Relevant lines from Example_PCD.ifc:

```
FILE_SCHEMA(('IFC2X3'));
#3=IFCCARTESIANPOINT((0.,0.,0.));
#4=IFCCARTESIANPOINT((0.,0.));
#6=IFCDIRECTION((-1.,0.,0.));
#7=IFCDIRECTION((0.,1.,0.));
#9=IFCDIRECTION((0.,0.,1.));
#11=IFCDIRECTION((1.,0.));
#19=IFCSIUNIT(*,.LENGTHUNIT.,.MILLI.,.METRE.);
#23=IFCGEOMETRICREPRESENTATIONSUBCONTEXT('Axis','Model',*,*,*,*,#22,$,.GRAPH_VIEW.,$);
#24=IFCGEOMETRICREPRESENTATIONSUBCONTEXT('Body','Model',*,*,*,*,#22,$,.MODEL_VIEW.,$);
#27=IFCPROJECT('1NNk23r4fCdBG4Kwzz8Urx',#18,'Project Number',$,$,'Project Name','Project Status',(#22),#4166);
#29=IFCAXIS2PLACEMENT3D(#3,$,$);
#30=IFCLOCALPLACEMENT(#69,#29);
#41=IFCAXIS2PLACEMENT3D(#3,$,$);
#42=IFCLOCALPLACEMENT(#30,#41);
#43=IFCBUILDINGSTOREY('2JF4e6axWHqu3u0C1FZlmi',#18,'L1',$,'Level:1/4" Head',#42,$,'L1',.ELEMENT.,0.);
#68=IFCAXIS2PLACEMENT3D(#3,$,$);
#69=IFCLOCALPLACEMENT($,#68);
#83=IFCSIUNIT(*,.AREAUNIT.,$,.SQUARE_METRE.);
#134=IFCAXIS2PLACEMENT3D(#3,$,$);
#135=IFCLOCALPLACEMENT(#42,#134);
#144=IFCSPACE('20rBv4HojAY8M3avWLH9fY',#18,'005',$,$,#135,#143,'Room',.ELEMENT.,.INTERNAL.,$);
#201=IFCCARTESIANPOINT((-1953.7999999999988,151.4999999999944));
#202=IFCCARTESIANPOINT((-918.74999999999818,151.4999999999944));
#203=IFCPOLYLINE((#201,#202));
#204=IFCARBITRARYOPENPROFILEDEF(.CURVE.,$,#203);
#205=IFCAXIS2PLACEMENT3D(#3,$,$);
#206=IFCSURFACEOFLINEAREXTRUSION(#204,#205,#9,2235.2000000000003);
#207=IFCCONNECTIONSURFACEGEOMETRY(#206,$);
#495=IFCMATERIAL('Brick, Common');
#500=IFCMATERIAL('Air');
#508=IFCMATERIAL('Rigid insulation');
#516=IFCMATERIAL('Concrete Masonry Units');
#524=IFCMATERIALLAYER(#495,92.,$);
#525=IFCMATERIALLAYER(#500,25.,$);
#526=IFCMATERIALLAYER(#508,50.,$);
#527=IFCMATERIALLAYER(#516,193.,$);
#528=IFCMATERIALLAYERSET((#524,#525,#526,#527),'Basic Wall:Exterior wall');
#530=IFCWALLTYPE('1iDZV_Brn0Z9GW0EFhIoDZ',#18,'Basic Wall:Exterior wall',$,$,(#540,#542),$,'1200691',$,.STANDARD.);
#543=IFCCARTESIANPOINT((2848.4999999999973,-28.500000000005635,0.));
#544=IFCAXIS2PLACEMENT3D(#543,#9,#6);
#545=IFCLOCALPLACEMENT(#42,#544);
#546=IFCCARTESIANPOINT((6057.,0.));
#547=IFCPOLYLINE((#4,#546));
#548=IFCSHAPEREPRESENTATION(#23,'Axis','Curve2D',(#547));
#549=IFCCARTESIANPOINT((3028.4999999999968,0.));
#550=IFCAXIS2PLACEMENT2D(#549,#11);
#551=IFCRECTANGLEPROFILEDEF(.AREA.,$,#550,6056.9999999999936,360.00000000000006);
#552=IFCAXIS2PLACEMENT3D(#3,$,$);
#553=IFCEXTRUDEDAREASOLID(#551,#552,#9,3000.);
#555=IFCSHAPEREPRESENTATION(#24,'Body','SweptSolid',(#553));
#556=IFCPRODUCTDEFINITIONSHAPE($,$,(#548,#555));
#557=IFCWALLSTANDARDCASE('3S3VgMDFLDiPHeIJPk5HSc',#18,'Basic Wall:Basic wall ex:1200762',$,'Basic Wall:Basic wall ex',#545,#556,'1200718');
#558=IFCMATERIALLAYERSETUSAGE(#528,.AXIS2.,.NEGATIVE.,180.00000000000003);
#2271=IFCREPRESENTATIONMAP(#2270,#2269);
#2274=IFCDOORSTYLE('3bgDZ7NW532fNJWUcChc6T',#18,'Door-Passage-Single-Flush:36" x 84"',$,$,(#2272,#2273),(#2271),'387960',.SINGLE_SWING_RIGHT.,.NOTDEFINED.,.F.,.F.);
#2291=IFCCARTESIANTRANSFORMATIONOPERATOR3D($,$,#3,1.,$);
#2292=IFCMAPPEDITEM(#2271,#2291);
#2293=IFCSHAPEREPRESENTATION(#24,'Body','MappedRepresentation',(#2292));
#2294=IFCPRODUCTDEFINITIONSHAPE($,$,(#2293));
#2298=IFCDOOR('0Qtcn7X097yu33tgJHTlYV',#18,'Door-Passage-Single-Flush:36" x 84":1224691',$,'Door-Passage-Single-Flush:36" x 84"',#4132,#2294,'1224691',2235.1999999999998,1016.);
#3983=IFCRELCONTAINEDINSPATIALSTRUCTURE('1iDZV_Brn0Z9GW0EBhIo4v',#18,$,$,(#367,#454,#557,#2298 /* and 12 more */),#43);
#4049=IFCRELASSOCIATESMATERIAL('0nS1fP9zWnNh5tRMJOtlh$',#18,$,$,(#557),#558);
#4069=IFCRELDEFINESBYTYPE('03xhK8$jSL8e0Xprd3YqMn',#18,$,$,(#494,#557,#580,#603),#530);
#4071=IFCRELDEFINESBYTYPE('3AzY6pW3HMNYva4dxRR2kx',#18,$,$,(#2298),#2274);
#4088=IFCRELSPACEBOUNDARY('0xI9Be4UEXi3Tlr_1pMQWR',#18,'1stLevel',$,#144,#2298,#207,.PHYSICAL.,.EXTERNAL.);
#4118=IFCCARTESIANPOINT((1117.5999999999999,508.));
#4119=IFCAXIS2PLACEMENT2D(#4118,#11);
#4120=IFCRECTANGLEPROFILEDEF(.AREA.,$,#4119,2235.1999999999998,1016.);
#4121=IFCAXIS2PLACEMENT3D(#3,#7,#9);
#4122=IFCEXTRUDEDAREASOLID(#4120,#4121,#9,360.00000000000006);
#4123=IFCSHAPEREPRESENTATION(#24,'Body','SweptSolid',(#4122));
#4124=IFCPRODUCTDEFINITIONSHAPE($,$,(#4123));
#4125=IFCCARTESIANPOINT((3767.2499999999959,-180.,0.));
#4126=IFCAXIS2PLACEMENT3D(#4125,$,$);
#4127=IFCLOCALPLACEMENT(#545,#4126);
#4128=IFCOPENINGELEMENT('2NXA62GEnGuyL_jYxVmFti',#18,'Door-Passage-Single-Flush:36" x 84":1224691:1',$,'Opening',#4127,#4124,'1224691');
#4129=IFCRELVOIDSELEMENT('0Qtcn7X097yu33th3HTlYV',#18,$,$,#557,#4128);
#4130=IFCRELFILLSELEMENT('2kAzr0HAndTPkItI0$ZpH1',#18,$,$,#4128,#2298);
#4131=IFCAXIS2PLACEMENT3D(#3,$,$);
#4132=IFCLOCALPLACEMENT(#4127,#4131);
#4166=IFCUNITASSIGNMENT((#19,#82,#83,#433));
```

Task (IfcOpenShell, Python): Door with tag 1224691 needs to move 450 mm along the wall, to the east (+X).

```python
import numpy as np
import ifcopenshell
import ifcopenshell.api.geometry
import ifcopenshell.util.placement

model = ifcopenshell.open("Example_PCD.ifc")

door = model.by_id(2298)
opening = door.FillsVoids[0].RelatingOpeningElement
wall = opening.VoidsElements[0].RelatingBuildingElement

wall_matrix = ifcopenshell.util.placement.get_local_placement(wall.ObjectPlacement)
shift = wall_matrix[:3, 0] * -450.0
before = ifcopenshell.util.placement.get_local_placement(door.ObjectPlacement)[:3, 3].copy()

# The door is placed relative to its opening, so it follows when the opening moves.
matrix = ifcopenshell.util.placement.get_local_placement(opening.ObjectPlacement)
matrix[:3, 3] += shift
ifcopenshell.api.geometry.edit_object_placement(
    model, product=opening, matrix=matrix, is_si=False, should_transform_children=True
)

# Space boundary surfaces are stored in each space's coordinates; move them too.
for rel in door.ProvidesBoundaries:
    if not rel.ConnectionGeometry:
        continue
    surface = rel.ConnectionGeometry.SurfaceOnRelatingElement
    space_matrix = ifcopenshell.util.placement.get_local_placement(rel.RelatingSpace.ObjectPlacement)
    point = np.array(surface.Position.Location.Coordinates) + space_matrix[:3, :3].T @ shift
    surface.Position = model.createIfcAxis2Placement3D(
        model.createIfcCartesianPoint(point.tolist()), surface.Position.Axis, surface.Position.RefDirection
    )

after = ifcopenshell.util.placement.get_local_placement(door.ObjectPlacement)[:3, 3]
print("door moved by", (after - before).round(3) + 0.0)

model.write("Example_PCD_v2.ifc")
```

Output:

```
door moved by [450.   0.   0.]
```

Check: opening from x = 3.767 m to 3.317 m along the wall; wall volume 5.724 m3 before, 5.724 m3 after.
